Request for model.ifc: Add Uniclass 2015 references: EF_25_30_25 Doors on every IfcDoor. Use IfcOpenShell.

First a look at what the model holds.

```python
import ifcopenshell

model = ifcopenshell.open("model.ifc")
print(model.schema)
print("classifications:", [c.Name for c in model.by_type("IfcClassification")])
for ifc_class in ("IfcDoor", "IfcRoof", "IfcStair", "IfcWall", "IfcWindow"):
    print(ifc_class, len(model.by_type(ifc_class)))
```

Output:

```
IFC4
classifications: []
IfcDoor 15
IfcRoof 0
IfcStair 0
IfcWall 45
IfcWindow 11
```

```python
import ifcopenshell
import ifcopenshell.api.classification

model = ifcopenshell.open("model.ifc")

system = ifcopenshell.api.classification.add_classification(model, classification="Uniclass 2015")

codes = {
    "IfcDoor": ("EF_25_30_25", "Doors"),
}
for ifc_class, (code, name) in codes.items():
    products = model.by_type(ifc_class)
    ifcopenshell.api.classification.add_reference(
        model, products=products, classification=system, identification=code, name=name
    )
    print(code, len(products))

model.write("model_v2.ifc")
```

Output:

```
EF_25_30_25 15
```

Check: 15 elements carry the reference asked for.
